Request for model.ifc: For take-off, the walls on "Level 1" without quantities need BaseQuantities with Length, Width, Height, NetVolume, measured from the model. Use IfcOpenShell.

First a look at what the model holds.

```python
import ifcopenshell
import ifcopenshell.util.element
import ifcopenshell.util.unit

model = ifcopenshell.open("model.ifc")
print(model.schema)
for unit_type in ("LENGTHUNIT", "AREAUNIT", "VOLUMEUNIT"):
    print(unit_type, ifcopenshell.util.unit.calculate_unit_scale(model, unit_type))
storey = next(s for s in model.by_type("IfcBuildingStorey") if s.Name == "Level 1")
walls = [e for e in ifcopenshell.util.element.get_decomposition(storey) if e.is_a("IfcWall")]
for e in sorted(walls, key=lambda e: e.id()):
    print(e.id(), e.is_a(), e.Name, list(ifcopenshell.util.element.get_psets(e, qtos_only=True)), sep=" | ")
```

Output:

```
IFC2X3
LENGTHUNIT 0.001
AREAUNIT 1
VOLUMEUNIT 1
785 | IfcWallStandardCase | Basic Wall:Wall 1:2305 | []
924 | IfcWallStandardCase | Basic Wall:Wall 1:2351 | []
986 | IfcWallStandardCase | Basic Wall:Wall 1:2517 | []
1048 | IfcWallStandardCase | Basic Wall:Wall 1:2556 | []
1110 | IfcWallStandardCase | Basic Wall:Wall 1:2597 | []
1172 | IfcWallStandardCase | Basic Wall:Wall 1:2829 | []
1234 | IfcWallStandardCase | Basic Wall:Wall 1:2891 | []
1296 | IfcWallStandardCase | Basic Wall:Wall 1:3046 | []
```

```python
import ifcopenshell
import ifcopenshell.api.pset
import ifcopenshell.geom
import ifcopenshell.util.element
import ifcopenshell.util.shape
import ifcopenshell.util.unit

model = ifcopenshell.open("model.ifc")
unit_scale = ifcopenshell.util.unit.calculate_unit_scale(model)
volume_scale = ifcopenshell.util.unit.calculate_unit_scale(model, "VOLUMEUNIT")
settings = ifcopenshell.geom.settings()

storey = next(s for s in model.by_type("IfcBuildingStorey") if s.Name == "Level 1")
walls = [e for e in ifcopenshell.util.element.get_decomposition(storey) if e.is_a("IfcWall")]

for e in sorted(walls, key=lambda e: e.id()):
    if ifcopenshell.util.element.get_psets(e, qtos_only=True, should_inherit=False):
        continue
    # Geometry comes back in metres, in the element's own axes.
    shape = ifcopenshell.geom.create_shape(settings, e)
    values = {
        "Length": ifcopenshell.util.shape.get_x(shape.geometry) / unit_scale,
        "Width": ifcopenshell.util.shape.get_y(shape.geometry) / unit_scale,
        "Height": ifcopenshell.util.shape.get_z(shape.geometry) / unit_scale,
        "NetVolume": ifcopenshell.util.shape.get_volume(shape.geometry) / volume_scale,
    }
    qto = ifcopenshell.api.pset.add_qto(model, product=e, name="BaseQuantities")
    ifcopenshell.api.pset.edit_qto(model, qto=qto, properties=values)
    print(e.id(), {k: round(v, 3) for k, v in values.items()})

model.write("model_v2.ifc")
```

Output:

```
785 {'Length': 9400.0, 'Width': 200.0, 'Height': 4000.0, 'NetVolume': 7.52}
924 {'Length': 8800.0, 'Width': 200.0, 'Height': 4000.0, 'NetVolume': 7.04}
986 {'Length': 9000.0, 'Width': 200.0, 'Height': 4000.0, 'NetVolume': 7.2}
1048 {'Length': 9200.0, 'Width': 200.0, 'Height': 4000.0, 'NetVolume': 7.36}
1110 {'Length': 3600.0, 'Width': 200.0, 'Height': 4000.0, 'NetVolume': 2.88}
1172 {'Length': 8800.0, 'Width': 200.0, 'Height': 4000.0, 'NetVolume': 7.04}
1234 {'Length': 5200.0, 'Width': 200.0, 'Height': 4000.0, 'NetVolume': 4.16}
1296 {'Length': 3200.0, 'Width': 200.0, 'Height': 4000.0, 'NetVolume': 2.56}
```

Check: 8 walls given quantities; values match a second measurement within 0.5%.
